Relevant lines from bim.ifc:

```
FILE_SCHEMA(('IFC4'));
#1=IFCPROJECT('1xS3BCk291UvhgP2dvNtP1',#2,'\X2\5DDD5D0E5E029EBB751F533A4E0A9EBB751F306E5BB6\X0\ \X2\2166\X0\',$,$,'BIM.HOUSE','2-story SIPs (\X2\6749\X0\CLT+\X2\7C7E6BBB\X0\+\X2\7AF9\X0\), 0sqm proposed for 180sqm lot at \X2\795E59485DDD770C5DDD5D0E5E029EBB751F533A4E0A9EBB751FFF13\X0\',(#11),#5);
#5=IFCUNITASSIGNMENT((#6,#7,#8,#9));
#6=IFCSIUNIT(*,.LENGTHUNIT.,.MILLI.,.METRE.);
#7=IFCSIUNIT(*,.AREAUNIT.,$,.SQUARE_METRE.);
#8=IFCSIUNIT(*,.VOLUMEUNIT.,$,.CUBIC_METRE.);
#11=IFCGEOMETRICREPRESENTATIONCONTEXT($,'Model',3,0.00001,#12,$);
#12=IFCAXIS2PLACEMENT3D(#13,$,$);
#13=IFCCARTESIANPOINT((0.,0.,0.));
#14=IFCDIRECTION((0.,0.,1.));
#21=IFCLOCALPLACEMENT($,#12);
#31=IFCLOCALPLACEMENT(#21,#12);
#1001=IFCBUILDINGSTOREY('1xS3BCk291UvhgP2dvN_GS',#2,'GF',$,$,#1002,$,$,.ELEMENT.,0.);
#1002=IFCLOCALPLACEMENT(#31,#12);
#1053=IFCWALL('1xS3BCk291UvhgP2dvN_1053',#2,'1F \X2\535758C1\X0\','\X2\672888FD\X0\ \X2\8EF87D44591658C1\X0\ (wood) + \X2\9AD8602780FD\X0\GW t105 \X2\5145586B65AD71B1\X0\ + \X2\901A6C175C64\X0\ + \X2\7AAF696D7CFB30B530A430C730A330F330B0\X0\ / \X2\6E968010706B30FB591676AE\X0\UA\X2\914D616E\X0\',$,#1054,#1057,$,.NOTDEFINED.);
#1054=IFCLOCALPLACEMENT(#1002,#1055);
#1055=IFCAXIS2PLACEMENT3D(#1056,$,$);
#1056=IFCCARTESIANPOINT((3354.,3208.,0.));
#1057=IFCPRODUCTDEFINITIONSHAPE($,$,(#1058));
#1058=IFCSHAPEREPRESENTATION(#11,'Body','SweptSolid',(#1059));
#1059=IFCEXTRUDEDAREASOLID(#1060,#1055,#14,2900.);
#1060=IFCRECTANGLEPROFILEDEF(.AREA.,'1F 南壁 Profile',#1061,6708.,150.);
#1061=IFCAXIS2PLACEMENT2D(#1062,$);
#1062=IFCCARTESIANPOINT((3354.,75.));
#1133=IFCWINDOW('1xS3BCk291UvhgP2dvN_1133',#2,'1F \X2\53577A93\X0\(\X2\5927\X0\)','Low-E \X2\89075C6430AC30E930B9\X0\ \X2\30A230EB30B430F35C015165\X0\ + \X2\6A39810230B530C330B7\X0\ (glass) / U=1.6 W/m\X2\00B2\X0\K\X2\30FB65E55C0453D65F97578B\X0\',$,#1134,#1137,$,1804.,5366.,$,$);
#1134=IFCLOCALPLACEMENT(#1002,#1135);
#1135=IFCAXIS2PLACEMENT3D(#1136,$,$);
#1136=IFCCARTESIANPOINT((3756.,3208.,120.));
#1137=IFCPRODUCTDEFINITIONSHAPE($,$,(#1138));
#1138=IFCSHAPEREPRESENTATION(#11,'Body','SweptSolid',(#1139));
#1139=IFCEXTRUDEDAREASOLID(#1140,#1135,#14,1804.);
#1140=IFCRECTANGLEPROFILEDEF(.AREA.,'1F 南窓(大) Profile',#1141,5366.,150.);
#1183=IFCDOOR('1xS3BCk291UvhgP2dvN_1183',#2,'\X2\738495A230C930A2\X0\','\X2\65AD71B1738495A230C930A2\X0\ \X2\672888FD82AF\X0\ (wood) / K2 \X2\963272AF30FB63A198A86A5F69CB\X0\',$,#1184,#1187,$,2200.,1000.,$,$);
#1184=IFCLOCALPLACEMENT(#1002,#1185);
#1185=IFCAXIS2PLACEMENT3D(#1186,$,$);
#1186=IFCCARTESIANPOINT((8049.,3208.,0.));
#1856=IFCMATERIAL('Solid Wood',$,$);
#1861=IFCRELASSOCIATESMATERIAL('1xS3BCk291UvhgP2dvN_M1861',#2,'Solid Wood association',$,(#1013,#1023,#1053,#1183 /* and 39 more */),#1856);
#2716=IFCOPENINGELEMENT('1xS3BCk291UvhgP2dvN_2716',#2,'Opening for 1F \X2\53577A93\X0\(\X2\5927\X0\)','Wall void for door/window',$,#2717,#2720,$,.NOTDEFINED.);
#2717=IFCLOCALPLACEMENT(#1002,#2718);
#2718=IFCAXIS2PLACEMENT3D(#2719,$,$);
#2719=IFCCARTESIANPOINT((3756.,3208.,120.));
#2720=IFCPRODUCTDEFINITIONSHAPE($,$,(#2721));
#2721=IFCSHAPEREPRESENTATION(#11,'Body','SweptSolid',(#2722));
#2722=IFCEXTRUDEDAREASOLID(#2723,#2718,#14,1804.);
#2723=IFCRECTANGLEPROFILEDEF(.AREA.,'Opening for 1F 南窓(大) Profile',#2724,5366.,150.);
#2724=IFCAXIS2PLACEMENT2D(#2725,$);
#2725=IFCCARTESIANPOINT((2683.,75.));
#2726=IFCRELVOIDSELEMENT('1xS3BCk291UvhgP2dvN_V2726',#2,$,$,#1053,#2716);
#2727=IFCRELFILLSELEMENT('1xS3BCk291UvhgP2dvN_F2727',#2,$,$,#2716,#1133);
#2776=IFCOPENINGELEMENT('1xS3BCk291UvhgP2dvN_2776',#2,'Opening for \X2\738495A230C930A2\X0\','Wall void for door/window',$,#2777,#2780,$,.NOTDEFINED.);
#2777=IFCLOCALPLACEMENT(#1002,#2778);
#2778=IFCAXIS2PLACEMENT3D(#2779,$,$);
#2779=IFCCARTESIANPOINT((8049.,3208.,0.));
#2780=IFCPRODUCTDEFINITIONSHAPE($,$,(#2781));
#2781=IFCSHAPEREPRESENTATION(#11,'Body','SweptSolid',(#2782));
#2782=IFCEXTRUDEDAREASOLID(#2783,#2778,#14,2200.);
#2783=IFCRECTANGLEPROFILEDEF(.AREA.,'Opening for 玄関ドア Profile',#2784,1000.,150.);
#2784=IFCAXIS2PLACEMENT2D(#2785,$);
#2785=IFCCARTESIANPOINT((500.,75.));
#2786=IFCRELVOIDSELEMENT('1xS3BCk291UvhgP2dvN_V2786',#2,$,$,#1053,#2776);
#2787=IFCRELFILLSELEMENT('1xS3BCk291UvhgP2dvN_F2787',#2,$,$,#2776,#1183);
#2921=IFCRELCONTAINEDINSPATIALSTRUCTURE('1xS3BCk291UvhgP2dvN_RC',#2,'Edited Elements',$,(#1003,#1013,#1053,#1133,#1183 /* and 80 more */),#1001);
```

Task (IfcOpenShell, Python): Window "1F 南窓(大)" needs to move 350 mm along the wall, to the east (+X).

```python
import ifcopenshell
import ifcopenshell.api.geometry
import ifcopenshell.util.placement
import ifcopenshell.util.unit

model = ifcopenshell.open("bim.ifc")
unit_scale = ifcopenshell.util.unit.calculate_unit_scale(model)

window = model.by_guid("1xS3BCk291UvhgP2dvN_1133")
opening = window.FillsVoids[0].RelatingOpeningElement
wall = opening.VoidsElements[0].RelatingBuildingElement

wall_matrix = ifcopenshell.util.placement.get_local_placement(wall.ObjectPlacement)
shift = wall_matrix[:3, 0] * 0.35 / unit_scale
before = ifcopenshell.util.placement.get_local_placement(window.ObjectPlacement)[:3, 3].copy()

# The window is not placed relative to its opening, so move both.
for product in (opening, window):
    matrix = ifcopenshell.util.placement.get_local_placement(product.ObjectPlacement)
    matrix[:3, 3] += shift
    ifcopenshell.api.geometry.edit_object_placement(model, product=product, matrix=matrix, is_si=False)

after = ifcopenshell.util.placement.get_local_placement(window.ObjectPlacement)[:3, 3]
print("window moved by", (after - before).round(3) + 0.0)

model.write("bim_edited.ifc")
```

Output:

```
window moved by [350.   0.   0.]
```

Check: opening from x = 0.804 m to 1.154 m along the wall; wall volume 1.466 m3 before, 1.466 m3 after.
